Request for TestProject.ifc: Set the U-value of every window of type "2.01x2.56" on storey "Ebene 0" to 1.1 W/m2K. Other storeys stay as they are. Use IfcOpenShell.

First a look at what the model holds.

```python
import ifcopenshell
import ifcopenshell.util.element

model = ifcopenshell.open("TestProject.ifc")
print(model.schema)
storey = next(s for s in model.by_type("IfcBuildingStorey") if s.Name == "Ebene 0")
windows = [e for e in ifcopenshell.util.element.get_decomposition(storey) if e.is_a("IfcWindow")]
seen = {}
for e in windows:
    element_type = ifcopenshell.util.element.get_type(e)
    key = (element_type.Name if element_type != e and element_type else None, ifcopenshell.util.element.get_pset(e, "Pset_WindowCommon", "ThermalTransmittance"))
    seen[key] = seen.get(key, 0) + 1
for (name, value), count in sorted(seen.items(), key=str):
    print(count, "x", name, "|", value)
```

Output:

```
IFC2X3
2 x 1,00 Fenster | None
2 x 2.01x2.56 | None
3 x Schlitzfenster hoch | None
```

```python
import ifcopenshell
import ifcopenshell.api.pset
import ifcopenshell.util.element

model = ifcopenshell.open("TestProject.ifc")

storey = next(s for s in model.by_type("IfcBuildingStorey") if s.Name == "Ebene 0")
windows = [e for e in ifcopenshell.util.element.get_decomposition(storey) if e.is_a("IfcWindow")]

count = 0
for e in windows:
    element_type = ifcopenshell.util.element.get_type(e)
    if element_type in (None, e) or element_type.Name != "2.01x2.56":
        continue
    # add_pset returns the element's existing set when there is one.
    pset = ifcopenshell.api.pset.add_pset(model, product=e, name="Pset_WindowCommon")
    ifcopenshell.api.pset.edit_pset(model, pset=pset, properties={"ThermalTransmittance": 1.1})
    count += 1

print(count, "windows updated")

model.write("TestProject_rev.ifc")
```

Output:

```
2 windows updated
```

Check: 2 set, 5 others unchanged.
